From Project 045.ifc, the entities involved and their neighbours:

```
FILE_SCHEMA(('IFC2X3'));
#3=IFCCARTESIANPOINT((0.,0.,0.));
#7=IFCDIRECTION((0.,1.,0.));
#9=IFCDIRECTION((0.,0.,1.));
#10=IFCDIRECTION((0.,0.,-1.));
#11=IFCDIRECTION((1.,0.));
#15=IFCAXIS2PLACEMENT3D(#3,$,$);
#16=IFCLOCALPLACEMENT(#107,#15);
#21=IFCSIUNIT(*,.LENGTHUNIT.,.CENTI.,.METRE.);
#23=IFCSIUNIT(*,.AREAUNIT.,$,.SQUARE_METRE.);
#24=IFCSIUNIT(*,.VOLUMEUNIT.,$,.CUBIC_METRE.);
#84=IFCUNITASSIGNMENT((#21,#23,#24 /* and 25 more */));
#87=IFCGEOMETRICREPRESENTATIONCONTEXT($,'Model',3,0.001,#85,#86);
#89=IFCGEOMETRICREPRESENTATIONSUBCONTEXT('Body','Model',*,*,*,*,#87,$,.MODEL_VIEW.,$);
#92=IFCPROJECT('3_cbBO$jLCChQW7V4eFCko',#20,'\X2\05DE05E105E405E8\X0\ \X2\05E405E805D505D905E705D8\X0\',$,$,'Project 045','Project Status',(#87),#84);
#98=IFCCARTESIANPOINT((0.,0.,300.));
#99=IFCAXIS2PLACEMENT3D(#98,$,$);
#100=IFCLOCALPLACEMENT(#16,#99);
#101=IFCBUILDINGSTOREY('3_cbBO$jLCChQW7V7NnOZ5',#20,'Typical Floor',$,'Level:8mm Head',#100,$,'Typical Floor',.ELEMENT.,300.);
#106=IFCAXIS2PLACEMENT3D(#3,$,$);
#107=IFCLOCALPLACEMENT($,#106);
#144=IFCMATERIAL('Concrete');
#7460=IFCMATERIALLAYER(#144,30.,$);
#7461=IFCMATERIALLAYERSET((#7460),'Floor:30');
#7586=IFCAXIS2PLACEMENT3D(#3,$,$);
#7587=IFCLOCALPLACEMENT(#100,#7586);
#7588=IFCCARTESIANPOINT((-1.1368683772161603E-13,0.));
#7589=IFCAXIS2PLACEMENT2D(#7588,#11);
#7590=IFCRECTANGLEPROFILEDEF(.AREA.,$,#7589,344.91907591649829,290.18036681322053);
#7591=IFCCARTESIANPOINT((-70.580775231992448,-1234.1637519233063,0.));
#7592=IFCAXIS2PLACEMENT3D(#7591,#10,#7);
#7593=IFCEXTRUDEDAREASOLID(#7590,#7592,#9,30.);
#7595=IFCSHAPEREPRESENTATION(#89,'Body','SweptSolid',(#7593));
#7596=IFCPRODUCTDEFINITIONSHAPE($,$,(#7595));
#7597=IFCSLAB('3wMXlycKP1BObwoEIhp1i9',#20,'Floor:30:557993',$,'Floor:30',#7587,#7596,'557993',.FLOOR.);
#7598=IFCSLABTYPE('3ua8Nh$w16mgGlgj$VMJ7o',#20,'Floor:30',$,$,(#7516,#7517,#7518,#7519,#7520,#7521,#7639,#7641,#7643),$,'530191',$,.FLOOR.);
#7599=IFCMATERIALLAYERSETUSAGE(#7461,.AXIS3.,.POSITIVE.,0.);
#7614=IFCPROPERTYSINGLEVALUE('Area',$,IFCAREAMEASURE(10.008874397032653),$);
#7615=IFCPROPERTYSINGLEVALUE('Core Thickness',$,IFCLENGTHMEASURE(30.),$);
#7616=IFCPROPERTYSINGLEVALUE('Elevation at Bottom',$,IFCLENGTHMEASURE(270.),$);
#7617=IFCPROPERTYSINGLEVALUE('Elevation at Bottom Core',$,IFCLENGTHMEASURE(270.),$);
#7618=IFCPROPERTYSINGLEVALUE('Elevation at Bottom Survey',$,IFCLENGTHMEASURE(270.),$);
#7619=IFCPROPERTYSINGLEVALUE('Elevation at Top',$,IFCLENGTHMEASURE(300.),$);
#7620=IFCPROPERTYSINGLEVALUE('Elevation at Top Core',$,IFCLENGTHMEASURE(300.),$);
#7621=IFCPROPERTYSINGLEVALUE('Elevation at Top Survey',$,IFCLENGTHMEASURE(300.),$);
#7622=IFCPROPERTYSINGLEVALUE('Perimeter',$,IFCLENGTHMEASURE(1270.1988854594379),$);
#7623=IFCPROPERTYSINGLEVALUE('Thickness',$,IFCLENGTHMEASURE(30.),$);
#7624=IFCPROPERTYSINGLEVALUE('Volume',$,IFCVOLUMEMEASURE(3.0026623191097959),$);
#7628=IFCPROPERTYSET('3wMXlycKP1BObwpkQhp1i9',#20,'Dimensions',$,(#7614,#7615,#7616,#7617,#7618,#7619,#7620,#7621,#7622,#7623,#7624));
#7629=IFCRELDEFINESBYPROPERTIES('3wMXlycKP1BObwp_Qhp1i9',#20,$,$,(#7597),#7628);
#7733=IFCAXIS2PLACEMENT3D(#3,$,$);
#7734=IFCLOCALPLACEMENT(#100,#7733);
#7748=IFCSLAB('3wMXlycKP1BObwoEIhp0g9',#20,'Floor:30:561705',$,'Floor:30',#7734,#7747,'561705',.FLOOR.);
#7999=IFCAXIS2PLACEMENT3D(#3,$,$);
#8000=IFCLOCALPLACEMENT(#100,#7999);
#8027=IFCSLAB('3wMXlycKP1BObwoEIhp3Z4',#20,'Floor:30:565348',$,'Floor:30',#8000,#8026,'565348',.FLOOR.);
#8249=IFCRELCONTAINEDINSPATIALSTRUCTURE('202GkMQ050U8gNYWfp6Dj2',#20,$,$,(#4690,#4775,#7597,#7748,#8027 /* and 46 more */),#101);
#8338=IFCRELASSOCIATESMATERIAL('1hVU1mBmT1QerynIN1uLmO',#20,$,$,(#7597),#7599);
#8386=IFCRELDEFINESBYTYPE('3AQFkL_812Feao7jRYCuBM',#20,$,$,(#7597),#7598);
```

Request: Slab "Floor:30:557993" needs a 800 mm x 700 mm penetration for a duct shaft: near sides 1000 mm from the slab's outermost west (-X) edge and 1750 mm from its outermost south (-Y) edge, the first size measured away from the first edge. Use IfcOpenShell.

```python
import numpy as np
import ifcopenshell
import ifcopenshell.api.feature
import ifcopenshell.api.geometry
import ifcopenshell.api.pset
import ifcopenshell.api.root
import ifcopenshell.geom
import ifcopenshell.util.element
import ifcopenshell.util.placement
import ifcopenshell.util.representation
import ifcopenshell.util.shape
import ifcopenshell.util.unit

model = ifcopenshell.open("Project 045.ifc")
unit_scale = ifcopenshell.util.unit.calculate_unit_scale(model)
area_scale = ifcopenshell.util.unit.calculate_unit_scale(model, "AREAUNIT")
volume_scale = ifcopenshell.util.unit.calculate_unit_scale(model, "VOLUMEUNIT")
settings = ifcopenshell.geom.settings()


def volume(element):
    """Net volume in cubic metres, openings subtracted."""
    shape = ifcopenshell.geom.create_shape(settings, element)
    return ifcopenshell.util.shape.get_volume(shape.geometry)


slab = model.by_guid("3wMXlycKP1BObwoEIhp1i9")
before = volume(slab)

# Extent in the slab's own axes, in metres. The edges named are its -X and -Y sides.
slab_shape = ifcopenshell.geom.create_shape(settings, slab)
vertices = ifcopenshell.util.shape.get_vertices(slab_shape.geometry)
x_min, y_min, bottom = vertices.min(axis=0)
top = vertices[:, 2].max()

opening = ifcopenshell.api.root.create_entity(model, ifc_class="IfcOpeningElement", name="Duct shaft opening")
context = ifcopenshell.util.representation.get_context(model, "Model", "Body", "MODEL_VIEW")
width, depth = 0.8, 0.7
outline = [(0.0, 0.0), (width, 0.0), (width, depth), (0.0, depth), (0.0, 0.0)]
# Overshoot both faces by 50 mm so the cut is clean.
shape = ifcopenshell.api.geometry.add_slab_representation(
    model, context=context, depth=top - bottom + 0.1, polyline=outline
)
ifcopenshell.api.geometry.assign_representation(model, product=opening, representation=shape)

matrix = ifcopenshell.util.placement.get_local_placement(slab.ObjectPlacement)
matrix[:, 3] = matrix @ np.append(np.array([x_min + 1, y_min + 1.75, bottom - 0.05]) / unit_scale, 1.0)
ifcopenshell.api.geometry.edit_object_placement(model, product=opening, matrix=matrix, is_si=False)
ifcopenshell.api.feature.add_feature(model, feature=opening, element=slab)

after = volume(slab)

# Update the slab's stored quantities.
pset = model.by_id(ifcopenshell.util.element.get_pset(slab, "Dimensions", should_inherit=False)["id"])
ifcopenshell.api.pset.edit_pset(model, pset=pset, properties={
    "Area": model.create_entity("IfcAreaMeasure", after / (top - bottom) / area_scale),
    "Volume": model.create_entity("IfcVolumeMeasure", after / volume_scale),
})

print(f"slab volume {before:.3f} -> {after:.3f} m3")

model.write("Project 045_edited.ifc")
```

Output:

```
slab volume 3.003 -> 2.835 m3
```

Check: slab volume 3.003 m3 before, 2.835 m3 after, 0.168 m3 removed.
